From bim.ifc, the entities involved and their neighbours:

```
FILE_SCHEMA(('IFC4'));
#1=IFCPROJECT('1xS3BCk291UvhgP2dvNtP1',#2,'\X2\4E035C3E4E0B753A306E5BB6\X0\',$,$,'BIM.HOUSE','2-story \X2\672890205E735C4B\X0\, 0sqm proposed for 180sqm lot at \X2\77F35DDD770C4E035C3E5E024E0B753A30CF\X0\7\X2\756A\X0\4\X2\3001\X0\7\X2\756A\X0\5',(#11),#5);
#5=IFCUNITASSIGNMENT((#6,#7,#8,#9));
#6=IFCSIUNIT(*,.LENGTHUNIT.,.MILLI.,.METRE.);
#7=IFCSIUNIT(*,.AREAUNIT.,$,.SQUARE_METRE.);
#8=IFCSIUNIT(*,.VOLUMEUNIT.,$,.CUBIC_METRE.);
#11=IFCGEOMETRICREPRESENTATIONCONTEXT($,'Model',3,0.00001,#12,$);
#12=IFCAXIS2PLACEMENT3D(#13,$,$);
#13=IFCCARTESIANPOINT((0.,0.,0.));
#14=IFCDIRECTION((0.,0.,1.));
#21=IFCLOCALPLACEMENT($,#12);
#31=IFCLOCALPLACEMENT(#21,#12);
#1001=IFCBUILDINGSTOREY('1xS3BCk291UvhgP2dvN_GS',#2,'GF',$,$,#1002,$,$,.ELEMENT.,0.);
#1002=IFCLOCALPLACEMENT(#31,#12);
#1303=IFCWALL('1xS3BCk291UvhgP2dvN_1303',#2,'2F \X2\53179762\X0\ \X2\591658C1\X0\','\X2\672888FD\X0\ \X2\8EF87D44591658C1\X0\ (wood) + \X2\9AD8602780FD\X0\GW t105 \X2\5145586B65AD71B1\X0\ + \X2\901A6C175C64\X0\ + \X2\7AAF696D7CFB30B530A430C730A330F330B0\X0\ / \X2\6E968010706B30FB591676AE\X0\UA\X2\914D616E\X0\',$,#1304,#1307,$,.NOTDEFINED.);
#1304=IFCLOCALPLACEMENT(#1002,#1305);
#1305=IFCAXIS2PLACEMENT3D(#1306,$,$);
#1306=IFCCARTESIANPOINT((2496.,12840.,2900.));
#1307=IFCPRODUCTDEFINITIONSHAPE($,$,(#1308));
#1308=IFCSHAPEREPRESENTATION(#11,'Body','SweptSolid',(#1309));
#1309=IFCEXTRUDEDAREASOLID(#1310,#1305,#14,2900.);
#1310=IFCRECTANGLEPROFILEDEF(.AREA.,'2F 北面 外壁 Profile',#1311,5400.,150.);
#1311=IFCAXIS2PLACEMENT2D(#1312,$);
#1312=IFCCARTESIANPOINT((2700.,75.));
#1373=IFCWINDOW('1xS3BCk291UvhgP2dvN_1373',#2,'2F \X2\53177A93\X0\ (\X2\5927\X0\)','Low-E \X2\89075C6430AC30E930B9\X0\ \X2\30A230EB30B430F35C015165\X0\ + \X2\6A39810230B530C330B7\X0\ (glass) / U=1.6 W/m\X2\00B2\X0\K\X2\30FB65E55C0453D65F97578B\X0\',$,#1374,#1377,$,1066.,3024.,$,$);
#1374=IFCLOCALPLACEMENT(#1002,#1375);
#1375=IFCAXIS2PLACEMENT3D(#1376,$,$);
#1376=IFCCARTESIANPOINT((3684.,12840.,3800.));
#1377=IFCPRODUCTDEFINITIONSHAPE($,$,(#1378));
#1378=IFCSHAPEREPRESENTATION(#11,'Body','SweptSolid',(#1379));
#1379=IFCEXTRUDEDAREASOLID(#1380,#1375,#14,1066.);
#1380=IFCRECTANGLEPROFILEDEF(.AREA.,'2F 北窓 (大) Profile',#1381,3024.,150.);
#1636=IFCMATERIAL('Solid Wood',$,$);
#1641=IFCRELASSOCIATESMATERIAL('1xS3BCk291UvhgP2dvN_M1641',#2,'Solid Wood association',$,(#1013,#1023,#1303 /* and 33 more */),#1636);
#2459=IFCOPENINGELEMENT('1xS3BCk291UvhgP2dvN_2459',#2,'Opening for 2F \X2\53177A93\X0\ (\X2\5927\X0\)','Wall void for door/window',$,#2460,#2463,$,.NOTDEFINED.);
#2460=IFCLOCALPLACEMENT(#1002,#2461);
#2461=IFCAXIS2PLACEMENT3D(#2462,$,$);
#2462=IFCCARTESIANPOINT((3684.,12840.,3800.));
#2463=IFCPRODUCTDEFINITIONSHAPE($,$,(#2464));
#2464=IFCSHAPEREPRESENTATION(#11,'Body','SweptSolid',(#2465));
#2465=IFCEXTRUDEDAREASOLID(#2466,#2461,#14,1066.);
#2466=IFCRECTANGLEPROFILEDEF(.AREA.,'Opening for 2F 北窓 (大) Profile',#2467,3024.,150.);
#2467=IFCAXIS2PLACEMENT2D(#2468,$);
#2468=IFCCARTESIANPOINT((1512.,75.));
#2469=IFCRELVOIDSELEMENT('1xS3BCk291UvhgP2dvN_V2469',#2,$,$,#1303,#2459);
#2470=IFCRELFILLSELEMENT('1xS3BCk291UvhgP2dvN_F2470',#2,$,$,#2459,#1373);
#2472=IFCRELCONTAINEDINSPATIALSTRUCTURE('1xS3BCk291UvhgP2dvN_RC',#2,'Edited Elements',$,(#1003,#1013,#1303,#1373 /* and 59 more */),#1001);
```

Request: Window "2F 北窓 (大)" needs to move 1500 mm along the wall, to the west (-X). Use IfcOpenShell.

```python
import ifcopenshell
import ifcopenshell.api.geometry
import ifcopenshell.util.placement
import ifcopenshell.util.unit

model = ifcopenshell.open("bim.ifc")
unit_scale = ifcopenshell.util.unit.calculate_unit_scale(model)

window = model.by_guid("1xS3BCk291UvhgP2dvN_1373")
opening = window.FillsVoids[0].RelatingOpeningElement
wall = opening.VoidsElements[0].RelatingBuildingElement

wall_matrix = ifcopenshell.util.placement.get_local_placement(wall.ObjectPlacement)
shift = wall_matrix[:3, 0] * -1.5 / unit_scale
before = ifcopenshell.util.placement.get_local_placement(window.ObjectPlacement)[:3, 3].copy()

# The window is not placed relative to its opening, so move both.
for product in (opening, window):
    matrix = ifcopenshell.util.placement.get_local_placement(product.ObjectPlacement)
    matrix[:3, 3] += shift
    ifcopenshell.api.geometry.edit_object_placement(model, product=product, matrix=matrix, is_si=False)

after = ifcopenshell.util.placement.get_local_placement(window.ObjectPlacement)[:3, 3]
print("window moved by", (after - before).round(3) + 0.0)

model.write("bim_v2.ifc")
```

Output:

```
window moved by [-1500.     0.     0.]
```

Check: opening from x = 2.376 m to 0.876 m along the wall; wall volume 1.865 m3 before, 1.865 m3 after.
